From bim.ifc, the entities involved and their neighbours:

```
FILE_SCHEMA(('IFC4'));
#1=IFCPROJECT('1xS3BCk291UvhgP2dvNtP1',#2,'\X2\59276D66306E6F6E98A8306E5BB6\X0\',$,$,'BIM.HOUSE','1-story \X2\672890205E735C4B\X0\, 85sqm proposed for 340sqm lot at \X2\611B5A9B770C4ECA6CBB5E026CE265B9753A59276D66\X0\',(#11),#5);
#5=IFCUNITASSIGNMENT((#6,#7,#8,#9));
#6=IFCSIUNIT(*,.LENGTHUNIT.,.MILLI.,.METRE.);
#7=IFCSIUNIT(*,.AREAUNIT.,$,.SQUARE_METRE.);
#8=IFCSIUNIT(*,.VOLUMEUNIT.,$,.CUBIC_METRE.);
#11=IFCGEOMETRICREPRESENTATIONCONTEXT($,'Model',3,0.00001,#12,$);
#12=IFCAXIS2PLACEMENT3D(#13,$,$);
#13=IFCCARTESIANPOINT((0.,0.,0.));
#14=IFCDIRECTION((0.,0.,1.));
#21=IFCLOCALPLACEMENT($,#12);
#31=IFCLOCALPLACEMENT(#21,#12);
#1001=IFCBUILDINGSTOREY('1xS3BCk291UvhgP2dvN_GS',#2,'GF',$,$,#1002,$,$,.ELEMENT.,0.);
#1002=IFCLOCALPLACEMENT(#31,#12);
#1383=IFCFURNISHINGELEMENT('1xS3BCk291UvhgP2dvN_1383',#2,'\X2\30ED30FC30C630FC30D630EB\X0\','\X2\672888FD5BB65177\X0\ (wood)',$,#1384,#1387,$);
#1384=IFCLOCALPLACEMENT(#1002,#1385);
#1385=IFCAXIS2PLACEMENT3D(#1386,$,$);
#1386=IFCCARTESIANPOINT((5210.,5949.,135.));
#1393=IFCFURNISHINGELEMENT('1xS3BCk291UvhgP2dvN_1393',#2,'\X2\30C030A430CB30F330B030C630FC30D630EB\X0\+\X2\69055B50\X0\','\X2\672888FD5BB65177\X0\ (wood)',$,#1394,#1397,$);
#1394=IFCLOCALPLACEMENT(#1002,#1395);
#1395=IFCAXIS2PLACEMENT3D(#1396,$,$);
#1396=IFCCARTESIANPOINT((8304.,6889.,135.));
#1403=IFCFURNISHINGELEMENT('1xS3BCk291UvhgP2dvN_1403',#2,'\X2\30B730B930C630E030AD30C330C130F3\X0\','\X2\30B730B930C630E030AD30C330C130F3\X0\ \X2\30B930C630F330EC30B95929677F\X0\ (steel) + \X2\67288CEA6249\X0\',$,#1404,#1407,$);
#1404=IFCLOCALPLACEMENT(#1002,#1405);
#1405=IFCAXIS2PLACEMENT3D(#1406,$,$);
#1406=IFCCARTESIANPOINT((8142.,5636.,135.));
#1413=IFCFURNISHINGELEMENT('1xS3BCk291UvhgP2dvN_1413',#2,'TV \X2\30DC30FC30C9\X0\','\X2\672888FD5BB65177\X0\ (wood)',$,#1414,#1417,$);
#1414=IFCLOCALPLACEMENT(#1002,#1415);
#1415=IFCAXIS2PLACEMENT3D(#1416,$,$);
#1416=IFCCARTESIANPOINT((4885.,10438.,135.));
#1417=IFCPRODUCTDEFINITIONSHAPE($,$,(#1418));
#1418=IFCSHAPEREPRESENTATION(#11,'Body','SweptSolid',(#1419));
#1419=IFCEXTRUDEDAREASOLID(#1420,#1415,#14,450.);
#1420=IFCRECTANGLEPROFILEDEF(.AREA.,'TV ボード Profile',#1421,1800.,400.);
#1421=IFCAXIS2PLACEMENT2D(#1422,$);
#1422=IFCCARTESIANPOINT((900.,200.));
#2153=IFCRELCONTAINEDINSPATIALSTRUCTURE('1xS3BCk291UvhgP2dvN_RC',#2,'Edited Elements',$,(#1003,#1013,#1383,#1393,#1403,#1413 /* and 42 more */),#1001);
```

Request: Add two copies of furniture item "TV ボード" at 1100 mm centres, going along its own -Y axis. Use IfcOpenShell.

```python
import ifcopenshell
import ifcopenshell.api.geometry
import ifcopenshell.api.root
import ifcopenshell.util.element
import ifcopenshell.util.placement
import ifcopenshell.util.unit

model = ifcopenshell.open("bim.ifc")
unit_scale = ifcopenshell.util.unit.calculate_unit_scale(model)


def reuse_history(source, copy):
    """copy_class also copies each property set's owner history, people and application; keep the originals."""
    for rel in copy.IsDefinedBy:
        if rel.is_a("IfcRelDefinesByProperties") and (history := rel.RelatingPropertyDefinition.OwnerHistory):
            rel.RelatingPropertyDefinition.OwnerHistory = source.OwnerHistory
            ifcopenshell.util.element.remove_deep2(model, history)


source = model.by_guid("1xS3BCk291UvhgP2dvN_1413")
base = ifcopenshell.util.placement.get_local_placement(source.ObjectPlacement)
step = -base[:3, 1] * 1.1 / unit_scale

for i in range(1, 3):
    copy = ifcopenshell.api.root.copy_class(model, product=source)
    copy.Representation = ifcopenshell.util.element.copy_deep(
        model, source.Representation, exclude=["IfcGeometricRepresentationContext", "IfcRepresentationMap"]
    )
    reuse_history(source, copy)
    matrix = base.copy()
    matrix[:3, 3] += i * step
    print("added at", matrix[:3, 3].round(3) + 0.0)
    ifcopenshell.api.geometry.edit_object_placement(model, product=copy, matrix=matrix, is_si=False)

model.write("bim_updated.ifc")
```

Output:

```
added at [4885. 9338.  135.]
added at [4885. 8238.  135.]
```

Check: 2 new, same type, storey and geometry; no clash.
